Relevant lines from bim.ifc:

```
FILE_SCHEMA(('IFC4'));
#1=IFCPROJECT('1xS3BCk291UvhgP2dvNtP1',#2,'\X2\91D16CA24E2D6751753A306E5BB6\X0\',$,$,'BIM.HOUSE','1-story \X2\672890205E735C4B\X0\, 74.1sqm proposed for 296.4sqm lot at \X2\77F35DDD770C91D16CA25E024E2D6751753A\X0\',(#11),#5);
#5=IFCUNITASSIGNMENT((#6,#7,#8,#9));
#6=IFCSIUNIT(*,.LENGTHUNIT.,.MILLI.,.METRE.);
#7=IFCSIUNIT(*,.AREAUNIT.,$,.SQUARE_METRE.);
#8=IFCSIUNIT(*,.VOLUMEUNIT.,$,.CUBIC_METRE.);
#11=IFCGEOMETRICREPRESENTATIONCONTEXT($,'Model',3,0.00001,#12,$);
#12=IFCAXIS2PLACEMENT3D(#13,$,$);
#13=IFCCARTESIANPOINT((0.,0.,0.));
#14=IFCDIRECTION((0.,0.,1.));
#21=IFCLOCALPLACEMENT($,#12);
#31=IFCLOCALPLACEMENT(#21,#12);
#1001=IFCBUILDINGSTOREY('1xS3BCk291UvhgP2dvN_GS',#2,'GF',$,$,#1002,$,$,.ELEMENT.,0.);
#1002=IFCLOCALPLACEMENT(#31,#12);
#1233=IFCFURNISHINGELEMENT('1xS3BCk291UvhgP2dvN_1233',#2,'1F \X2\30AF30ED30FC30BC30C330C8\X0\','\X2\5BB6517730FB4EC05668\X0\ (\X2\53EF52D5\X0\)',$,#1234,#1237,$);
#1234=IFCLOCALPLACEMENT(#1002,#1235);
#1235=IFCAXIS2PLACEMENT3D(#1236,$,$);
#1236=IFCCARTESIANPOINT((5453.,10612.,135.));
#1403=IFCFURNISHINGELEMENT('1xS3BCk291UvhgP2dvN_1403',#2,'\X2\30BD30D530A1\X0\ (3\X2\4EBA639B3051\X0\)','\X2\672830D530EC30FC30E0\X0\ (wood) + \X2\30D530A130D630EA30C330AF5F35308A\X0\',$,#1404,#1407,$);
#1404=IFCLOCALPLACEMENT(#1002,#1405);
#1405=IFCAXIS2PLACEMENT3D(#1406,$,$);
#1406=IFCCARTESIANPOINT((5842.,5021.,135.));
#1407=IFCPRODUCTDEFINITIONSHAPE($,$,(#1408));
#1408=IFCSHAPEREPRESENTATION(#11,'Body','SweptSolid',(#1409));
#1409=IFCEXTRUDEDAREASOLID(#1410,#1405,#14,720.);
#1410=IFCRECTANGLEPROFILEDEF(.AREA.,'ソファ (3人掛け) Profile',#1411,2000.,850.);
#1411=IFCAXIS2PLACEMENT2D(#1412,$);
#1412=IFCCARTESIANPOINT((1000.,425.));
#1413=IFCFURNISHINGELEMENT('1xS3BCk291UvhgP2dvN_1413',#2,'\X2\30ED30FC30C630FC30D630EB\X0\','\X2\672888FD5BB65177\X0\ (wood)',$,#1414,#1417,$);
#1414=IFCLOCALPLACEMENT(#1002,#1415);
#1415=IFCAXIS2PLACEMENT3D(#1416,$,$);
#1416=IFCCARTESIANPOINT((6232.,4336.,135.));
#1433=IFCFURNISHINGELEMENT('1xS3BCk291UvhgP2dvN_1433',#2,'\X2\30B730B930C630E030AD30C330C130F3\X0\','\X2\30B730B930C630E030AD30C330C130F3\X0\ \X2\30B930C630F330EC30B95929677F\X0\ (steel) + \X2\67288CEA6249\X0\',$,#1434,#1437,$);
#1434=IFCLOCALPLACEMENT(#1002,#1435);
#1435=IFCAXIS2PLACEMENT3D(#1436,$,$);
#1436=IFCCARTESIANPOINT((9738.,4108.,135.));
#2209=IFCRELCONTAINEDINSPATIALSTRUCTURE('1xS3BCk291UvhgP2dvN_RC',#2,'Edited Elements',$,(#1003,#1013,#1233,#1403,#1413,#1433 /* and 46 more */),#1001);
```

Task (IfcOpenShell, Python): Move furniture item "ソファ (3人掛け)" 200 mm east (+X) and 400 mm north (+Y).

```python
import ifcopenshell
import ifcopenshell.api.geometry
import ifcopenshell.util.placement
import ifcopenshell.util.unit

model = ifcopenshell.open("bim.ifc")
unit_scale = ifcopenshell.util.unit.calculate_unit_scale(model)

item = model.by_guid("1xS3BCk291UvhgP2dvN_1403")
matrix = ifcopenshell.util.placement.get_local_placement(item.ObjectPlacement)
matrix[0, 3] += 0.2 / unit_scale
matrix[1, 3] += 0.4 / unit_scale
ifcopenshell.api.geometry.edit_object_placement(model, product=item, matrix=matrix, is_si=False)

print(ifcopenshell.util.placement.get_local_placement(item.ObjectPlacement).round(3) + 0.0)

model.write("bim_updated.ifc")
```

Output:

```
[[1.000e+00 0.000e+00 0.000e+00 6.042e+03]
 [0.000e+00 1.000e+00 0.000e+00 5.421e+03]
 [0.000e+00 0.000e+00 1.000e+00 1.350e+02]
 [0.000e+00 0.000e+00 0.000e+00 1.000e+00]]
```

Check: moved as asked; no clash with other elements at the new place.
